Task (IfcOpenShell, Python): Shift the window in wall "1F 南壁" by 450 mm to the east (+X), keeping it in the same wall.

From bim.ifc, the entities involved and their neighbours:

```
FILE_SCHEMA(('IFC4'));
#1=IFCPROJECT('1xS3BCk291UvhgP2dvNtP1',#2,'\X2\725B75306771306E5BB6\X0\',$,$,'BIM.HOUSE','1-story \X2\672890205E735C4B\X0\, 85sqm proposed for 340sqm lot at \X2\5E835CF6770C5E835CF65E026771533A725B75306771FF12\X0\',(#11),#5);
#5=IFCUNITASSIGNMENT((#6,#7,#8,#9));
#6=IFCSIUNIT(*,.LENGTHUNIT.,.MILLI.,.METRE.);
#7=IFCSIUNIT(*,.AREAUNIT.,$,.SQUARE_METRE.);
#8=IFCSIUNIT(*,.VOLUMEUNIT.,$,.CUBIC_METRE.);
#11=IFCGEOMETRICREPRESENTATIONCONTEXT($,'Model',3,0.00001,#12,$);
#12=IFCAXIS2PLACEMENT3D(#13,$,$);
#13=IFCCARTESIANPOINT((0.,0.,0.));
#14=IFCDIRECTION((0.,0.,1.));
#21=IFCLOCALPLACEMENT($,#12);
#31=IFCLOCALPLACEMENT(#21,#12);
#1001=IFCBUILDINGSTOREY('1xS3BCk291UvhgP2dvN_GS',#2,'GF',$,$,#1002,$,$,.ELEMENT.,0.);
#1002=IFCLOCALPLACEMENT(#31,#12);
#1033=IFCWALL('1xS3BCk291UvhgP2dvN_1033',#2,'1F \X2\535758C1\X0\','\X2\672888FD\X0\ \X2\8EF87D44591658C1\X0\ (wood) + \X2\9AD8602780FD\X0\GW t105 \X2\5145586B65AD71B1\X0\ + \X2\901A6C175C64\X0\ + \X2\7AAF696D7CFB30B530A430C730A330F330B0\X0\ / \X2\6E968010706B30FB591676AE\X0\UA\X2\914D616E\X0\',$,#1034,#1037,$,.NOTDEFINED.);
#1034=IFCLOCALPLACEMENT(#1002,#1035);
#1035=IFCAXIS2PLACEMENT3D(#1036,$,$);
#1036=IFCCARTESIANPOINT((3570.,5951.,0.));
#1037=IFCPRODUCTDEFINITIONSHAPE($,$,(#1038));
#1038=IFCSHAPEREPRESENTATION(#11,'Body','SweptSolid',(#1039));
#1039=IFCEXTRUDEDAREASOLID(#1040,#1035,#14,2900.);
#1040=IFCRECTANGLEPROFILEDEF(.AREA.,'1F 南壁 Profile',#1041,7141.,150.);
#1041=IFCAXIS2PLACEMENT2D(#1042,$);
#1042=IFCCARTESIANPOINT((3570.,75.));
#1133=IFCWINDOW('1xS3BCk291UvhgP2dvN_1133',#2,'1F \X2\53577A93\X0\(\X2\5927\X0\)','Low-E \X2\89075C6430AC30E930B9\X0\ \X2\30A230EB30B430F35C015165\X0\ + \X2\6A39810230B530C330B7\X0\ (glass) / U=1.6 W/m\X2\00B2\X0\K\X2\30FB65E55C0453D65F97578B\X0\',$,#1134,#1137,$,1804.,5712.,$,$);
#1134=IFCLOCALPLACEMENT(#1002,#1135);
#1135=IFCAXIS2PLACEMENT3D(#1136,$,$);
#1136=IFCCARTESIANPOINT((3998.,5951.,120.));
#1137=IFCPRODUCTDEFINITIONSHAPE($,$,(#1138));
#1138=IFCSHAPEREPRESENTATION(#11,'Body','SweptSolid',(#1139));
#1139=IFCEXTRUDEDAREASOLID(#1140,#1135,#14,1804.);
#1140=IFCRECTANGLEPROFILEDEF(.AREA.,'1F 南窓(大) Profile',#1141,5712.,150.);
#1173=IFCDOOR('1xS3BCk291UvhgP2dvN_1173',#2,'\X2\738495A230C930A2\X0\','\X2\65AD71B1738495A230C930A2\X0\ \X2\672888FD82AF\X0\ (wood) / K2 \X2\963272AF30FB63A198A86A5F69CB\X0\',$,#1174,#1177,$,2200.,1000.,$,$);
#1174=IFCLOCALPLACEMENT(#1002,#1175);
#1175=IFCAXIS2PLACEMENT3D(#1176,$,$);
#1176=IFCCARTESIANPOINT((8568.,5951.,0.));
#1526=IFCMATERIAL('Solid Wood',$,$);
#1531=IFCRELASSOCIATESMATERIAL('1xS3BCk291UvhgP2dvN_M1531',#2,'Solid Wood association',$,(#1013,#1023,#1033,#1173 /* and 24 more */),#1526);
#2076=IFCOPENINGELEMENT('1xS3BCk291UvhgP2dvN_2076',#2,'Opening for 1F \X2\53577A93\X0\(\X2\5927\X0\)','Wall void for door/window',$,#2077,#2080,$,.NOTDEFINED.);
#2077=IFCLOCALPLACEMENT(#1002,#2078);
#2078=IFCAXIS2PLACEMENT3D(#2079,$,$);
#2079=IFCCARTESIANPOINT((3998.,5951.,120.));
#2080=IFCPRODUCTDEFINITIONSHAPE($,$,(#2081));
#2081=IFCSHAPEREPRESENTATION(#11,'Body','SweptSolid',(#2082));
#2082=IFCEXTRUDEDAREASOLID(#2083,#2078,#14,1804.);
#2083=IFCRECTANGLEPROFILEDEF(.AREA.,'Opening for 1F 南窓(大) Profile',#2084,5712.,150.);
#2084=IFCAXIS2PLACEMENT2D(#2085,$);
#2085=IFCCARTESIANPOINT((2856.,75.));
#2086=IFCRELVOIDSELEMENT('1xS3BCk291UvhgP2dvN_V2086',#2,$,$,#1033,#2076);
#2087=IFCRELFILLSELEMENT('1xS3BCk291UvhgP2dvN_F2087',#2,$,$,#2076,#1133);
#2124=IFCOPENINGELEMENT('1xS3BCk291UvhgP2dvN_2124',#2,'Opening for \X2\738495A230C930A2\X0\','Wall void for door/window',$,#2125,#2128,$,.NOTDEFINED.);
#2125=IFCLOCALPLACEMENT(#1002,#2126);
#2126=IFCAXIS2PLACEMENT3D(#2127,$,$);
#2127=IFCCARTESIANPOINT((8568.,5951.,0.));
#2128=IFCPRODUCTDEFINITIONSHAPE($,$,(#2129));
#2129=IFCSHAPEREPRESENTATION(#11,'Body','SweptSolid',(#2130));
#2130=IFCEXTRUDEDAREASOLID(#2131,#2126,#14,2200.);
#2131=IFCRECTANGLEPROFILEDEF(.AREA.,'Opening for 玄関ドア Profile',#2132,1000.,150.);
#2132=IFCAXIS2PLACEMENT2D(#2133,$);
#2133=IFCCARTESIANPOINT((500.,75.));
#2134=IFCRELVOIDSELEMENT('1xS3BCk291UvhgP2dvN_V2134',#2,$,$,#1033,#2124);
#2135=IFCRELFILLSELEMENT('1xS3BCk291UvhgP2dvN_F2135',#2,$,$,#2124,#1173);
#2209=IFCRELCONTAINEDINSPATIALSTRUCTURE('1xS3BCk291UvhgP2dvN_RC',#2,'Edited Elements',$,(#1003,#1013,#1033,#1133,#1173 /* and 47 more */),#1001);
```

```python
import ifcopenshell
import ifcopenshell.api.geometry
import ifcopenshell.util.placement
import ifcopenshell.util.unit

model = ifcopenshell.open("bim.ifc")
unit_scale = ifcopenshell.util.unit.calculate_unit_scale(model)

window = model.by_guid("1xS3BCk291UvhgP2dvN_1133")
opening = window.FillsVoids[0].RelatingOpeningElement
wall = opening.VoidsElements[0].RelatingBuildingElement

wall_matrix = ifcopenshell.util.placement.get_local_placement(wall.ObjectPlacement)
shift = wall_matrix[:3, 0] * 0.45 / unit_scale
before = ifcopenshell.util.placement.get_local_placement(window.ObjectPlacement)[:3, 3].copy()

# The window is not placed relative to its opening, so move both.
for product in (opening, window):
    matrix = ifcopenshell.util.placement.get_local_placement(product.ObjectPlacement)
    matrix[:3, 3] += shift
    ifcopenshell.api.geometry.edit_object_placement(model, product=product, matrix=matrix, is_si=False)

after = ifcopenshell.util.placement.get_local_placement(window.ObjectPlacement)[:3, 3]
print("window moved by", (after - before).round(3) + 0.0)

model.write("bim-out.ifc")
```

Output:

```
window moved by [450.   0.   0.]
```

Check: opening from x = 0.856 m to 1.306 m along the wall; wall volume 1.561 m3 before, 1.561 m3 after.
